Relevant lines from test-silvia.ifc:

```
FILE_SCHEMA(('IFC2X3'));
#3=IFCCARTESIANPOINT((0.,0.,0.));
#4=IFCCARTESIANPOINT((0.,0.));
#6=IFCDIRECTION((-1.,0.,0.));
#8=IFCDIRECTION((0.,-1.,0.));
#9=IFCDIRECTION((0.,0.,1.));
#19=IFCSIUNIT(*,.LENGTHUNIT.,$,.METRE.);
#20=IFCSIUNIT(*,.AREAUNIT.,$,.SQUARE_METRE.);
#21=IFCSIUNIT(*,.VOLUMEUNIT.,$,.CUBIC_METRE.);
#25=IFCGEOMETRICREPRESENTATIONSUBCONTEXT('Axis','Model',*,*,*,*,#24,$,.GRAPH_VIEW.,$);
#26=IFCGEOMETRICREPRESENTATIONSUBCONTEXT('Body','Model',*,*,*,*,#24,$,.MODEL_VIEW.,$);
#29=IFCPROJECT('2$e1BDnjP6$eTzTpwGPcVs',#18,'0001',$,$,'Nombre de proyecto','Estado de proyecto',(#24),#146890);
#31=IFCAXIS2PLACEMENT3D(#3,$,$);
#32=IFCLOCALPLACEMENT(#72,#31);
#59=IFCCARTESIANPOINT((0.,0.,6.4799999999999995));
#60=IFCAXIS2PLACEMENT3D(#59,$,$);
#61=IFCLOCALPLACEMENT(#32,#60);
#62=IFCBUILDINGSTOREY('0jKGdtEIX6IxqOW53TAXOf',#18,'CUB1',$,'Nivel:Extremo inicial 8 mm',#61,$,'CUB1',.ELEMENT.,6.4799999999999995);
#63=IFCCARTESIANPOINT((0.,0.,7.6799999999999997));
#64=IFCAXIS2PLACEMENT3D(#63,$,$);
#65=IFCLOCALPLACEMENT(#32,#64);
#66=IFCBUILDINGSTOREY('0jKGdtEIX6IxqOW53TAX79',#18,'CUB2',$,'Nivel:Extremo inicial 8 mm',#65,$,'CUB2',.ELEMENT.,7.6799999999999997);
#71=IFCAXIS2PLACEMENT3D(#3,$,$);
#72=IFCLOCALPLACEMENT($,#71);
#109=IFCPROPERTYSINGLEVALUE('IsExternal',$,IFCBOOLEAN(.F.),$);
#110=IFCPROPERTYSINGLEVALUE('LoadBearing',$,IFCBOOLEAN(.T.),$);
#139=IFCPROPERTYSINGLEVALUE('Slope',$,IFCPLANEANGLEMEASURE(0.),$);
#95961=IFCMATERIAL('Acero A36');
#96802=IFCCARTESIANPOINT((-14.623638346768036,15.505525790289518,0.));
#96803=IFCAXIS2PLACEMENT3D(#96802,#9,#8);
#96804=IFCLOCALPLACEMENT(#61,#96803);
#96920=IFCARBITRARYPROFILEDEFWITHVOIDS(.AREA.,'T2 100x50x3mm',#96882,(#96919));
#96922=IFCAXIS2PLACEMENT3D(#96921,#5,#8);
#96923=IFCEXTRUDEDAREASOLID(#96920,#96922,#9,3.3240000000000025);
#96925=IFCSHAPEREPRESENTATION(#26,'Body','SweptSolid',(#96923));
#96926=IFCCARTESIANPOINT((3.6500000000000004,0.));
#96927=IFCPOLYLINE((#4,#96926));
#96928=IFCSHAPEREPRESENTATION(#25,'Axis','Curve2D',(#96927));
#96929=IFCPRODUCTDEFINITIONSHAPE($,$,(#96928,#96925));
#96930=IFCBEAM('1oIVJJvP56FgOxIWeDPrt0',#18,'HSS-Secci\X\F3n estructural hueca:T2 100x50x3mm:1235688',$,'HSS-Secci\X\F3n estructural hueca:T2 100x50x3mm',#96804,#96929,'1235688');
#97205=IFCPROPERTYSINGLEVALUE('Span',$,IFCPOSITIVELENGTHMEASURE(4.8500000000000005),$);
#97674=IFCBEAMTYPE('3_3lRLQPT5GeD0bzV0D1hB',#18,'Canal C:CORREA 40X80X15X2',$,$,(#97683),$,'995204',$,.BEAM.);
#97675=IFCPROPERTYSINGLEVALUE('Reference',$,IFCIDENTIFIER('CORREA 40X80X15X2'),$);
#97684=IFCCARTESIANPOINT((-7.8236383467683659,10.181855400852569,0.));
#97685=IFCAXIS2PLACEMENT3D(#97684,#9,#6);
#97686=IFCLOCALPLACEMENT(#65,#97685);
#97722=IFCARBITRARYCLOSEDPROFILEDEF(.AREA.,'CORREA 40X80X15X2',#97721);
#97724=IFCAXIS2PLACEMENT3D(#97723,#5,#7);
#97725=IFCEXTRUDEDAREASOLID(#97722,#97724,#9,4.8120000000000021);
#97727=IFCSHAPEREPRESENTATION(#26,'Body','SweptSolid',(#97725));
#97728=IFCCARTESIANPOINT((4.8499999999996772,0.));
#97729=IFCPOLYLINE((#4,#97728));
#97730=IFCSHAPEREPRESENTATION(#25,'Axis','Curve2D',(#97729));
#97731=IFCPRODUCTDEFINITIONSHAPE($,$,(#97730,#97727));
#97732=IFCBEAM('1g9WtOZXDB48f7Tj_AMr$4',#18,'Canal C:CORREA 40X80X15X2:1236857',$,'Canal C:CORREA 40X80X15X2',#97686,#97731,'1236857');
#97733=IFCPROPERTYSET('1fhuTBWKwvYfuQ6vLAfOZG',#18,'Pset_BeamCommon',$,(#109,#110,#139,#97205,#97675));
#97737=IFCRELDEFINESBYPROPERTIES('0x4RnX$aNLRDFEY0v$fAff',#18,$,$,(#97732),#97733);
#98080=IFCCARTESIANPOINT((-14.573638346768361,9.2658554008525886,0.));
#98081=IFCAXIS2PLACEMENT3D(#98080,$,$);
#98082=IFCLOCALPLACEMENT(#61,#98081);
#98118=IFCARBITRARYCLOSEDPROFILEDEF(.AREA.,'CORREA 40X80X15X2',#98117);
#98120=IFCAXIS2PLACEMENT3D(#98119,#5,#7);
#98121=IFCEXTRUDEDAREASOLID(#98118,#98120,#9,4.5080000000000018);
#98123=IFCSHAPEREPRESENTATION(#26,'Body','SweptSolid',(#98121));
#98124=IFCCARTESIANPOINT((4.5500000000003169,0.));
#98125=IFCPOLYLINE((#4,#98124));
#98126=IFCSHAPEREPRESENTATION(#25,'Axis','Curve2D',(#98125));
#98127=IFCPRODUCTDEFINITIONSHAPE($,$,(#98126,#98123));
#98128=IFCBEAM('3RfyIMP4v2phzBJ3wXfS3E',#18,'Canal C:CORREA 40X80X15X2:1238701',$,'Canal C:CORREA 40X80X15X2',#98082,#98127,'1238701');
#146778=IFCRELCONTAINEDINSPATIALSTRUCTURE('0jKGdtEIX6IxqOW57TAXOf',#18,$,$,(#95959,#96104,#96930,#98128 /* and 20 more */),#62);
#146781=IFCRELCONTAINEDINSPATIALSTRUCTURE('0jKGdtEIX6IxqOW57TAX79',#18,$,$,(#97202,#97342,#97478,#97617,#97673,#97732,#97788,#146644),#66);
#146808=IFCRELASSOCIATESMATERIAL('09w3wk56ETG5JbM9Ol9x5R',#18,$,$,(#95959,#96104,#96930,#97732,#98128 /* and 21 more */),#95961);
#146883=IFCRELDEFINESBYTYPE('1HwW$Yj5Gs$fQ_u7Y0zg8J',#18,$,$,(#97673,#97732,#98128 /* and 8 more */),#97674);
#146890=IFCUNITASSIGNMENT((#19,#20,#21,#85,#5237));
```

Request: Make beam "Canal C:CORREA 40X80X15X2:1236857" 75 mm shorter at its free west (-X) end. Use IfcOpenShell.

```python
import numpy as np
import ifcopenshell
import ifcopenshell.api.pset
import ifcopenshell.util.element
import ifcopenshell.util.representation
import ifcopenshell.util.unit

model = ifcopenshell.open("test-silvia.ifc")
unit_scale = ifcopenshell.util.unit.calculate_unit_scale(model)

member = model.by_id(97732)
change = -0.075 / unit_scale

# The extrusion runs towards the end named, so only its depth changes.
body = ifcopenshell.util.representation.get_representation(member, "Model", "Body")
solid = body.Items[0]
old_length = solid.Depth
solid.Depth += change

# Move the axis end point with it.
axis = next(r for r in member.Representation.Representations if r.RepresentationIdentifier == "Axis").Items[0]
start, end = (np.array(p.Coordinates) for p in axis.Points)
end = end + (end - start) / np.linalg.norm(end - start) * change
point = model.createIfcCartesianPoint(end.tolist())
axis.Points = [axis.Points[0], point]

# Update the stored length and volume.
pset = model.by_id(ifcopenshell.util.element.get_pset(member, "Pset_BeamCommon", should_inherit=False)["id"])
ifcopenshell.api.pset.edit_pset(model, pset=pset, properties={
    "Span": model.create_entity("IfcPositiveLengthMeasure", solid.Depth),
})

print(f"length {old_length:g} -> {solid.Depth:g}")

model.write("test-silvia-out.ifc")
```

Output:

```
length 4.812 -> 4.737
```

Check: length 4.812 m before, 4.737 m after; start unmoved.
